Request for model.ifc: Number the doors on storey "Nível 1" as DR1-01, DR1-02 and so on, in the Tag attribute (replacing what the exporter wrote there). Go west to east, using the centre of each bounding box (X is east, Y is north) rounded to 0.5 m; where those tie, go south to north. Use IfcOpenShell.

First a look at what the model holds.

```python
import ifcopenshell
import ifcopenshell.util.element
import ifcopenshell.util.placement

model = ifcopenshell.open("model.ifc")
print(model.schema)
storey = next(s for s in model.by_type("IfcBuildingStorey") if s.Name == "Nível 1")
doors = [e for e in ifcopenshell.util.element.get_decomposition(storey) if e.is_a("IfcDoor")]
for e in sorted(doors, key=lambda e: e.id()):
    origin = ifcopenshell.util.placement.get_local_placement(e.ObjectPlacement)[:3, 3]
    print(e.id(), e.Tag, e.Name, origin.round(2) + 0.0, sep=" | ")
```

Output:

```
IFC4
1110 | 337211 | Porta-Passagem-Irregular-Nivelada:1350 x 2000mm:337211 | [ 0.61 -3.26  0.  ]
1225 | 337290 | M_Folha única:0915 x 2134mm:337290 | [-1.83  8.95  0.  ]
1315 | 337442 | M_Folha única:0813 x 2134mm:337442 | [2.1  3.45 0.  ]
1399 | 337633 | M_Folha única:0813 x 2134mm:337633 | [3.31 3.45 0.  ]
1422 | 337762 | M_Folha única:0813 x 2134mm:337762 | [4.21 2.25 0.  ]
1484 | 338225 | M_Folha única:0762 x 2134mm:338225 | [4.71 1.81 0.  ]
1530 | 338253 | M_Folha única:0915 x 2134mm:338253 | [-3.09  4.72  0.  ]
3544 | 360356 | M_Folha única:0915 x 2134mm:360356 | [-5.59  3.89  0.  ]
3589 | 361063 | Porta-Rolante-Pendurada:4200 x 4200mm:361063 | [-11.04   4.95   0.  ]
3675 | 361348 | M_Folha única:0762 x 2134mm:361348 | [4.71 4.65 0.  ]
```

```python
import ifcopenshell
import ifcopenshell.geom
import ifcopenshell.util.element
import ifcopenshell.util.shape

model = ifcopenshell.open("model.ifc")
settings = ifcopenshell.geom.settings()
settings.set("use-world-coords", True)


def centre(element):
    shape = ifcopenshell.geom.create_shape(settings, element)
    return ifcopenshell.util.shape.get_bbox_centroid(shape.geometry)


storey = next(s for s in model.by_type("IfcBuildingStorey") if s.Name == "Nível 1")
doors = [e for e in ifcopenshell.util.element.get_decomposition(storey) if e.is_a("IfcDoor")]

# Insertion points can sit at a corner or the storey origin, so sort by the geometry (in metres).
centres = {e: centre(e) for e in doors}
doors.sort(key=lambda e: (round(centres[e][0] / 0.5), centres[e][1]))

for i, e in enumerate(doors, start=1):
    number = f"DR1-{i:02d}"
    e.Tag = number
    print(e.id(), number)

model.write("model_updated.ifc")
```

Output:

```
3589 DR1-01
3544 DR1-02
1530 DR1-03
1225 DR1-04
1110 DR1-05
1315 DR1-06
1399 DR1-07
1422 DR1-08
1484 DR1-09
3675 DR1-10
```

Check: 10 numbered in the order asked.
